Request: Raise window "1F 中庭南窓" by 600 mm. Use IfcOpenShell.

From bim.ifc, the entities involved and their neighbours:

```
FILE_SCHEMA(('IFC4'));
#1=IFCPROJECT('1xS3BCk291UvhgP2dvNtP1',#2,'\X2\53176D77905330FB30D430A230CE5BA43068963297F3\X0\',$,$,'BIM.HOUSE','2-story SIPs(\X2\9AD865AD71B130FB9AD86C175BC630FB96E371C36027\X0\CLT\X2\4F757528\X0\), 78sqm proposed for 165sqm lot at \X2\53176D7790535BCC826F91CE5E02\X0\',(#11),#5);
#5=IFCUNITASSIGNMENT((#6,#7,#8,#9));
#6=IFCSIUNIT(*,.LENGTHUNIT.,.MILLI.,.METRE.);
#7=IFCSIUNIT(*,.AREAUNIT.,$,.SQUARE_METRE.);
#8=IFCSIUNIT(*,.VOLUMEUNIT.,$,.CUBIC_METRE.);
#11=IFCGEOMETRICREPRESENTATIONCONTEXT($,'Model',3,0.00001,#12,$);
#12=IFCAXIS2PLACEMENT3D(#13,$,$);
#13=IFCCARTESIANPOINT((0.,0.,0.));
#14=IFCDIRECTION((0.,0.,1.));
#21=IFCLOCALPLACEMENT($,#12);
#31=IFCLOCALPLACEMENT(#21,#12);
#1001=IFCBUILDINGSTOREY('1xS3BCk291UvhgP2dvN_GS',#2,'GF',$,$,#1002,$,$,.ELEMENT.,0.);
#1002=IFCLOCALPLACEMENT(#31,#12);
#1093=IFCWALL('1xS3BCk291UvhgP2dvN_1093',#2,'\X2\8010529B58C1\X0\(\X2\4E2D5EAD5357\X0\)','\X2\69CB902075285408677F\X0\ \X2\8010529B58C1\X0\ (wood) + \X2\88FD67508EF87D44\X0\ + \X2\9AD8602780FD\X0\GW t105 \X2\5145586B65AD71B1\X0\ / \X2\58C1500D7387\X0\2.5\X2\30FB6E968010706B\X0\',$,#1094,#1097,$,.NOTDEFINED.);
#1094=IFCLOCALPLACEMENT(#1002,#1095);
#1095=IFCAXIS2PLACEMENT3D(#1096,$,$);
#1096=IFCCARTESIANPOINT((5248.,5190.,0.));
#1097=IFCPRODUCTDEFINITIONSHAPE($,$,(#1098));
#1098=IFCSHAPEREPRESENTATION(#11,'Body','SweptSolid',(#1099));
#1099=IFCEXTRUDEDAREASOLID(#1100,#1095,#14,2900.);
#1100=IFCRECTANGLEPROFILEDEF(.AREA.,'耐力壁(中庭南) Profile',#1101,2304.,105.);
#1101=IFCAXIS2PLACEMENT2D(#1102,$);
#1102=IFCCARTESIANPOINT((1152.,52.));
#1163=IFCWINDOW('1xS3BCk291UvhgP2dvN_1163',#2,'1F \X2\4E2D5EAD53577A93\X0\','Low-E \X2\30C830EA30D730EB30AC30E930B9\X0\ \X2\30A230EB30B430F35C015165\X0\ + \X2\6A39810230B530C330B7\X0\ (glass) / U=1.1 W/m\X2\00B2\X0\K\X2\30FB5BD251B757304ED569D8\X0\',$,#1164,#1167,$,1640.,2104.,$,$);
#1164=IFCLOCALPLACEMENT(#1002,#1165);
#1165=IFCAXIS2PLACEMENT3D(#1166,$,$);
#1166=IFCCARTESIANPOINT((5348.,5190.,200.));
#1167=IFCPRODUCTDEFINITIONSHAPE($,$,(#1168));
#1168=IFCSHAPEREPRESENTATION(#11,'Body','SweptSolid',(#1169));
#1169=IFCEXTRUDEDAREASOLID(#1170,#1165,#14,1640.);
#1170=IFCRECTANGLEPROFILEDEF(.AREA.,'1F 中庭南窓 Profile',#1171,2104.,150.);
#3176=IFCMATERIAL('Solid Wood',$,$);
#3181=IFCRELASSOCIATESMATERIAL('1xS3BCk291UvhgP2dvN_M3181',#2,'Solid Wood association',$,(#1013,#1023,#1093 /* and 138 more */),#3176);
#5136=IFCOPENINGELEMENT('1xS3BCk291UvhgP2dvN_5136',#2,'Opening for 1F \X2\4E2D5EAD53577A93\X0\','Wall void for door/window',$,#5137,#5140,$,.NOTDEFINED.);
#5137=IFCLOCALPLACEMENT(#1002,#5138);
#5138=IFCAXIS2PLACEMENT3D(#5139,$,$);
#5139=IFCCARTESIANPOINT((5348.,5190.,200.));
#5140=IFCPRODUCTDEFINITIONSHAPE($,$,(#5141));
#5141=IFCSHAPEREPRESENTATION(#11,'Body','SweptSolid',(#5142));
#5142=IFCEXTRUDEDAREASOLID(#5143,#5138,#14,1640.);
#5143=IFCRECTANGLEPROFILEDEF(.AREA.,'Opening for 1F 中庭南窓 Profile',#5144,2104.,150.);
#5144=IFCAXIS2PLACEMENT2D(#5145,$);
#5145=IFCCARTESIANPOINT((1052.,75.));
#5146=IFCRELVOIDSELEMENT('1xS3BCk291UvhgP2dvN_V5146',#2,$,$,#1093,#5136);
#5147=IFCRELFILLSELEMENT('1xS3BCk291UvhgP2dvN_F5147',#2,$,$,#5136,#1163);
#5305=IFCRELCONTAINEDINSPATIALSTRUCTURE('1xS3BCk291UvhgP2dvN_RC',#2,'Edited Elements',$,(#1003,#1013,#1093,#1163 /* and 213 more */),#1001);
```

```python
import numpy as np
import ifcopenshell
import ifcopenshell.api.geometry
import ifcopenshell.util.placement
import ifcopenshell.util.unit

model = ifcopenshell.open("bim.ifc")
unit_scale = ifcopenshell.util.unit.calculate_unit_scale(model)

window = model.by_guid("1xS3BCk291UvhgP2dvN_1163")
opening = window.FillsVoids[0].RelatingOpeningElement
dz = 0.6 / unit_scale

shift = np.array([0.0, 0.0, dz])
# The window is not placed relative to its opening, so move both.
for product in (opening, window):
    matrix = ifcopenshell.util.placement.get_local_placement(product.ObjectPlacement)
    matrix[:3, 3] += shift
    ifcopenshell.api.geometry.edit_object_placement(model, product=product, matrix=matrix, is_si=False)

print(f"moved by {dz * unit_scale:+.3f} m")

model.write("bim_rev.ifc")
```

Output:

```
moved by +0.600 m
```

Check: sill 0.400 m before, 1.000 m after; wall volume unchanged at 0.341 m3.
